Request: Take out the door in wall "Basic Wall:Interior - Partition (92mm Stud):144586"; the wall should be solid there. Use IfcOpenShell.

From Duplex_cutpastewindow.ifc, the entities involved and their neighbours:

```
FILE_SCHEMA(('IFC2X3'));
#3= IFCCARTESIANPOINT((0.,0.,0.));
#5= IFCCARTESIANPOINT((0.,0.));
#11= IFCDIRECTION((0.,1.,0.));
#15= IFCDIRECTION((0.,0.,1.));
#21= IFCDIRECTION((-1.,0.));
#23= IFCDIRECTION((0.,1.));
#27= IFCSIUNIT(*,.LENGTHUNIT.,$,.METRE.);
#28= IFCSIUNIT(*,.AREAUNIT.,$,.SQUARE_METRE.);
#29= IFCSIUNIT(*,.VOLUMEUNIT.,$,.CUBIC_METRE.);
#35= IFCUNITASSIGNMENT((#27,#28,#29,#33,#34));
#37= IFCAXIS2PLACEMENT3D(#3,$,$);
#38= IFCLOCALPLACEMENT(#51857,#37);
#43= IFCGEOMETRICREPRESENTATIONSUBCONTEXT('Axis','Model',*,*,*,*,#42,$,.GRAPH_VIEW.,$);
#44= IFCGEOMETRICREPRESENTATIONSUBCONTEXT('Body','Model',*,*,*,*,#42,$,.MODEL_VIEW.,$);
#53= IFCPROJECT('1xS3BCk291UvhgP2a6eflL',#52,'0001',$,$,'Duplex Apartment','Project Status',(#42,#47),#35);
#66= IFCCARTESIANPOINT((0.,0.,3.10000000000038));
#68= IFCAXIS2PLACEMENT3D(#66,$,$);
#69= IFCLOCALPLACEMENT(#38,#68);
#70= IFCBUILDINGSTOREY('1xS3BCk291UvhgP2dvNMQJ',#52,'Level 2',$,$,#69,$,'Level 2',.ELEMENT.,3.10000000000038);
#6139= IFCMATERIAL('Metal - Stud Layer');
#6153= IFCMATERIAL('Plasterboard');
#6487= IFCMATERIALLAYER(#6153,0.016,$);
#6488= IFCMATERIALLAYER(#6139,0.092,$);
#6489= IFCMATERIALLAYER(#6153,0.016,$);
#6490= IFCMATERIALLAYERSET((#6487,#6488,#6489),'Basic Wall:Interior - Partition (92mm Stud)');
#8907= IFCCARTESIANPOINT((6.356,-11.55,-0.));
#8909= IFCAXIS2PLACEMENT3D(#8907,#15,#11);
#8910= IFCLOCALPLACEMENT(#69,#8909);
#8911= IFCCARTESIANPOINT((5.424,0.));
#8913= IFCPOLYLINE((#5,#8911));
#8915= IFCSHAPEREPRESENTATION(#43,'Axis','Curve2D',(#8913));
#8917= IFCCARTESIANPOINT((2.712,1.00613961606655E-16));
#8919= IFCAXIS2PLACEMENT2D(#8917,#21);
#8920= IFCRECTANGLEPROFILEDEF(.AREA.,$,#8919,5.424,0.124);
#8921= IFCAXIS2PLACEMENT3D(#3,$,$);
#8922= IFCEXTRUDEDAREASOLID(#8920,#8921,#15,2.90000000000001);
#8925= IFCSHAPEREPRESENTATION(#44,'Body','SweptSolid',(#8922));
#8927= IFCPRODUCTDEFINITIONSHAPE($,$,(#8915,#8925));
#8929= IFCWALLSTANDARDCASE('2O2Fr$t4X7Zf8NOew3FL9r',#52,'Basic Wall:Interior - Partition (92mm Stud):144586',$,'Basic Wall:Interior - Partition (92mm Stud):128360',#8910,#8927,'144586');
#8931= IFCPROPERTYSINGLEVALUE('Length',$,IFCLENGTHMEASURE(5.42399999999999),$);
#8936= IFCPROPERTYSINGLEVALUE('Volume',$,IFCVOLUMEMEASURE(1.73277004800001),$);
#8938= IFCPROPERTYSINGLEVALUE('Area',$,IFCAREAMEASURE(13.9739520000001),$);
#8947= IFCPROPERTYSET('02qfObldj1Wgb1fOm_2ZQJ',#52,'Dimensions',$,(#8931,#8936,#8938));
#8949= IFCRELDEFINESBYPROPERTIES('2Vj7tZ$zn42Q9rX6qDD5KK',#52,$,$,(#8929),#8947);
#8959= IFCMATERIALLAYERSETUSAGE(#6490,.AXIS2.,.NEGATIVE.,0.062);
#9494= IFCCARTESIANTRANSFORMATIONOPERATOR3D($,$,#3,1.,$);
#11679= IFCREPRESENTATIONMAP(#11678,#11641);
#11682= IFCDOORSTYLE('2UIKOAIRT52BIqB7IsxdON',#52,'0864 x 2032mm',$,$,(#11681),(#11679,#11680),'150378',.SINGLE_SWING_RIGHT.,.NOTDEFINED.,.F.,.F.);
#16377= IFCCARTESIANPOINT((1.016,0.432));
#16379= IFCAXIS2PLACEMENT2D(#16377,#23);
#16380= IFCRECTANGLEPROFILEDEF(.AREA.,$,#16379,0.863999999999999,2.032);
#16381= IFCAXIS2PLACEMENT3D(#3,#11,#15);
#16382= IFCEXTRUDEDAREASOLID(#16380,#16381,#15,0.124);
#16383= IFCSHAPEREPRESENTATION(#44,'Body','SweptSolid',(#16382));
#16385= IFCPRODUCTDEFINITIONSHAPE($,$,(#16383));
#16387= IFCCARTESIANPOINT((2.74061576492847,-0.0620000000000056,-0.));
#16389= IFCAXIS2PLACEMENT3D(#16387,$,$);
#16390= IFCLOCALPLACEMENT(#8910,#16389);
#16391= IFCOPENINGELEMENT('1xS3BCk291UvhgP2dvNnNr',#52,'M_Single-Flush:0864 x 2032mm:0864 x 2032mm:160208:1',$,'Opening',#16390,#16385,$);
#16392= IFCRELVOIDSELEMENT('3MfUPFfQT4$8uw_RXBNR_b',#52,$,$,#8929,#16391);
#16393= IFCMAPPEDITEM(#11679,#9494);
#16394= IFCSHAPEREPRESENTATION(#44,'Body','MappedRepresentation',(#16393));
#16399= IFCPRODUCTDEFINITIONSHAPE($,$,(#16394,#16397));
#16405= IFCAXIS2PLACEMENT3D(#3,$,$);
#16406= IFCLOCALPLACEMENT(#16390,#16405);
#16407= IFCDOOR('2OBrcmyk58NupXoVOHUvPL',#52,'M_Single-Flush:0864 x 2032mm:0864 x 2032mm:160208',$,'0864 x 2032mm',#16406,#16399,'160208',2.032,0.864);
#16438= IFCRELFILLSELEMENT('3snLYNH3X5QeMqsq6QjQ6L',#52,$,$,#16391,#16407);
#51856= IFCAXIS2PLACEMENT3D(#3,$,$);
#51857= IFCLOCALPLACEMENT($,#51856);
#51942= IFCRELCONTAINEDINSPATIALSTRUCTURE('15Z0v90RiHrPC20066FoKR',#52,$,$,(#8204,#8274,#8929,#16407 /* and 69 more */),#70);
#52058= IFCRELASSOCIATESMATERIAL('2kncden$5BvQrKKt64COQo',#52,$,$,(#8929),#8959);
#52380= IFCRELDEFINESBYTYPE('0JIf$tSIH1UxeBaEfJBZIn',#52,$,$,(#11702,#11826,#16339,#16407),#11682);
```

```python
import ifcopenshell
import ifcopenshell.api.feature
import ifcopenshell.api.pset
import ifcopenshell.api.root
import ifcopenshell.geom
import ifcopenshell.util.element
import ifcopenshell.util.shape
import ifcopenshell.util.unit

model = ifcopenshell.open("Duplex_cutpastewindow.ifc")
area_scale = ifcopenshell.util.unit.calculate_unit_scale(model, "AREAUNIT")
volume_scale = ifcopenshell.util.unit.calculate_unit_scale(model, "VOLUMEUNIT")
settings = ifcopenshell.geom.settings()


def volume(element):
    """Net volume in cubic metres, openings subtracted."""
    shape = ifcopenshell.geom.create_shape(settings, element)
    return ifcopenshell.util.shape.get_volume(shape.geometry)


door = model.by_id(16407)
opening = door.FillsVoids[0].RelatingOpeningElement
wall = opening.VoidsElements[0].RelatingBuildingElement
before = volume(wall)

ifcopenshell.api.root.remove_product(model, product=door)
ifcopenshell.api.feature.remove_feature(model, feature=opening)

after = volume(wall)
thickness = 0.124  # wall thickness in metres

# Update the wall's stored quantities.
pset = model.by_id(ifcopenshell.util.element.get_pset(wall, "Dimensions", should_inherit=False)["id"])
ifcopenshell.api.pset.edit_pset(model, pset=pset, properties={
    "Volume": model.create_entity("IfcVolumeMeasure", after / volume_scale),
    "Area": model.create_entity("IfcAreaMeasure", after / thickness / area_scale),
})

print(f"wall volume {before:.3f} -> {after:.3f} m3")

model.write("Duplex_cutpastewindow-out.ifc")
```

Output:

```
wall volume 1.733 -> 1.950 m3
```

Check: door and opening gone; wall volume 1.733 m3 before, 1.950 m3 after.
